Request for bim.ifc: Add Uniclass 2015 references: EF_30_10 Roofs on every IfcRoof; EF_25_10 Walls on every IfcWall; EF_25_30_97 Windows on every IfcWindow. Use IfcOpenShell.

First a look at what the model holds.

```python
import ifcopenshell

model = ifcopenshell.open("bim.ifc")
print(model.schema)
print("classifications:", [c.Name for c in model.by_type("IfcClassification")])
for ifc_class in ("IfcDoor", "IfcRoof", "IfcStair", "IfcWall", "IfcWindow"):
    print(ifc_class, len(model.by_type(ifc_class)))
```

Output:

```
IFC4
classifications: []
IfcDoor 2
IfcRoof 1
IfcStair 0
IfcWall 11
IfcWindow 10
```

```python
import ifcopenshell
import ifcopenshell.api.classification

model = ifcopenshell.open("bim.ifc")

system = ifcopenshell.api.classification.add_classification(model, classification="Uniclass 2015")

codes = {
    "IfcRoof": ("EF_30_10", "Roofs"),
    "IfcWall": ("EF_25_10", "Walls"),
    "IfcWindow": ("EF_25_30_97", "Windows"),
}
for ifc_class, (code, name) in codes.items():
    products = model.by_type(ifc_class)
    ifcopenshell.api.classification.add_reference(
        model, products=products, classification=system, identification=code, name=name
    )
    print(code, len(products))

model.write("bim-out.ifc")
```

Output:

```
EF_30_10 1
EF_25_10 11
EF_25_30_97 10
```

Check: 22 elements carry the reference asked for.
